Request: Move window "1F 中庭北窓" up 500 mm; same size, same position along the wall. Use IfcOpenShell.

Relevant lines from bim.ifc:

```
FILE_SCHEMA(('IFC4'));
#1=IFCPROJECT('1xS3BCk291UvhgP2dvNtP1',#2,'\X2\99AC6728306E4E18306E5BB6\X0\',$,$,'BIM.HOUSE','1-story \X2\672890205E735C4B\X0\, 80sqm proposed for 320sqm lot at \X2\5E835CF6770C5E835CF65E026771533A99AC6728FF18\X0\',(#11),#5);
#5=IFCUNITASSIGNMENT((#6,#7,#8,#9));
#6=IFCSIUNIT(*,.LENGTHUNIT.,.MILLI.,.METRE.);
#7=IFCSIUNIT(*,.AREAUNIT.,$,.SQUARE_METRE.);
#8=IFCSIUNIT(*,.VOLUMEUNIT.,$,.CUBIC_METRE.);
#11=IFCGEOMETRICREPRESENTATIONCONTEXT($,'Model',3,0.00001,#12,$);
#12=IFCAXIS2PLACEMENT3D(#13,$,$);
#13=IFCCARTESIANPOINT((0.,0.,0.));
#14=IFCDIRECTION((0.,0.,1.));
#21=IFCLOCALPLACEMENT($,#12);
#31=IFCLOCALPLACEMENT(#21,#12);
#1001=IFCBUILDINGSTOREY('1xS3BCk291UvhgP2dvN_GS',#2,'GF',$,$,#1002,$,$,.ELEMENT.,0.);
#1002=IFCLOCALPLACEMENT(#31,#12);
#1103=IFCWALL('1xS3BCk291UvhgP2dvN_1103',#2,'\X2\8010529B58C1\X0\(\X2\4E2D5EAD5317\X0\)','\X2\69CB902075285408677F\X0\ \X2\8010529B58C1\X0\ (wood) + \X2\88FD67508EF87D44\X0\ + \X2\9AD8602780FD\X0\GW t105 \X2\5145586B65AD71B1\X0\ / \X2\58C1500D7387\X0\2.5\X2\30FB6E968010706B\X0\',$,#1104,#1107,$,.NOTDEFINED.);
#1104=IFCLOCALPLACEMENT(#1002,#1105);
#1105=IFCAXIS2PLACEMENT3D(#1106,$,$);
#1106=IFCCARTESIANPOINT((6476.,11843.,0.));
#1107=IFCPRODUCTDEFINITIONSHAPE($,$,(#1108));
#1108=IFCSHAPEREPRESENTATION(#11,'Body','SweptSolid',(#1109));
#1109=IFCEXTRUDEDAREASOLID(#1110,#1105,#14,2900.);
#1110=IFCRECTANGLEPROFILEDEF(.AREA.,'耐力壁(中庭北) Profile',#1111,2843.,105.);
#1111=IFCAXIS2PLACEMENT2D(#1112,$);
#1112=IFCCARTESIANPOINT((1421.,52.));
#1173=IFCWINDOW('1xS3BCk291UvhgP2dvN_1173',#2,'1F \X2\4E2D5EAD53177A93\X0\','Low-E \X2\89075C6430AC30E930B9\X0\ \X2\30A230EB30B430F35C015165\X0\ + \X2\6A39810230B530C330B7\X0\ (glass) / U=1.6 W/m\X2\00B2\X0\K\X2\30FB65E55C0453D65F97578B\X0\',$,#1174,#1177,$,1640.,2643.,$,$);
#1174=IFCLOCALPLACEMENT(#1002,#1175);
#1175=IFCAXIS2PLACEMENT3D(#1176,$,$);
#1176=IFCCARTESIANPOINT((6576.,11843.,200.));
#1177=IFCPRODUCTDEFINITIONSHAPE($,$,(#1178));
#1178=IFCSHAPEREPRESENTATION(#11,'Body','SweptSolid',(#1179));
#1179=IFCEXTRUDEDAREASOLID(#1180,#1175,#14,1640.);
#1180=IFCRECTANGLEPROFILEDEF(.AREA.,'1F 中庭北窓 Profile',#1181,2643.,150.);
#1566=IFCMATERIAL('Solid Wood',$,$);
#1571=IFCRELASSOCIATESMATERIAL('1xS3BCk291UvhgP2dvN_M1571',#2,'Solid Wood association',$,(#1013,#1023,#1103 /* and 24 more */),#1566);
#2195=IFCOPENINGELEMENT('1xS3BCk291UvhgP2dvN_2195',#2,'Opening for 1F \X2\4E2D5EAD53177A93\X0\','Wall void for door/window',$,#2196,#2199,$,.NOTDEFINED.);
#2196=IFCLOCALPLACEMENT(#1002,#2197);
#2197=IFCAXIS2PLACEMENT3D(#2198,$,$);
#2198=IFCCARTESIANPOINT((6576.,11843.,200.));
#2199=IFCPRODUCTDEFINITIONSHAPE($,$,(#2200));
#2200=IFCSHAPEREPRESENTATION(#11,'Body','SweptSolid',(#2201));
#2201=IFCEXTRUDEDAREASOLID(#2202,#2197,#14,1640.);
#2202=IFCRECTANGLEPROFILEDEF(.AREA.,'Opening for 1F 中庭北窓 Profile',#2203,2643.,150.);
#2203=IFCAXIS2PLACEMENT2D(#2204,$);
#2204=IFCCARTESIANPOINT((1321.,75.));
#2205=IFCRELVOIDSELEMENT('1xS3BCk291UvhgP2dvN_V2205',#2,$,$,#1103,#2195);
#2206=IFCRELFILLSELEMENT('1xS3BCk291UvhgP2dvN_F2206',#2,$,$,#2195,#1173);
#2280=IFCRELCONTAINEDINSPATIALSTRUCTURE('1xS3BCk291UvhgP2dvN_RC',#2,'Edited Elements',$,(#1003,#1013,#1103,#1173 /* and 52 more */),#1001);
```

```python
import numpy as np
import ifcopenshell
import ifcopenshell.api.geometry
import ifcopenshell.util.placement
import ifcopenshell.util.unit

model = ifcopenshell.open("bim.ifc")
unit_scale = ifcopenshell.util.unit.calculate_unit_scale(model)

window = model.by_guid("1xS3BCk291UvhgP2dvN_1173")
opening = window.FillsVoids[0].RelatingOpeningElement
dz = 500.0

shift = np.array([0.0, 0.0, dz])
# The window is not placed relative to its opening, so move both.
for product in (opening, window):
    matrix = ifcopenshell.util.placement.get_local_placement(product.ObjectPlacement)
    matrix[:3, 3] += shift
    ifcopenshell.api.geometry.edit_object_placement(model, product=product, matrix=matrix, is_si=False)

print(f"moved by {dz * unit_scale:+.3f} m")

model.write("bim-out.ifc")
```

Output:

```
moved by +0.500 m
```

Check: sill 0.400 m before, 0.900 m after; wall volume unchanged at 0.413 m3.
